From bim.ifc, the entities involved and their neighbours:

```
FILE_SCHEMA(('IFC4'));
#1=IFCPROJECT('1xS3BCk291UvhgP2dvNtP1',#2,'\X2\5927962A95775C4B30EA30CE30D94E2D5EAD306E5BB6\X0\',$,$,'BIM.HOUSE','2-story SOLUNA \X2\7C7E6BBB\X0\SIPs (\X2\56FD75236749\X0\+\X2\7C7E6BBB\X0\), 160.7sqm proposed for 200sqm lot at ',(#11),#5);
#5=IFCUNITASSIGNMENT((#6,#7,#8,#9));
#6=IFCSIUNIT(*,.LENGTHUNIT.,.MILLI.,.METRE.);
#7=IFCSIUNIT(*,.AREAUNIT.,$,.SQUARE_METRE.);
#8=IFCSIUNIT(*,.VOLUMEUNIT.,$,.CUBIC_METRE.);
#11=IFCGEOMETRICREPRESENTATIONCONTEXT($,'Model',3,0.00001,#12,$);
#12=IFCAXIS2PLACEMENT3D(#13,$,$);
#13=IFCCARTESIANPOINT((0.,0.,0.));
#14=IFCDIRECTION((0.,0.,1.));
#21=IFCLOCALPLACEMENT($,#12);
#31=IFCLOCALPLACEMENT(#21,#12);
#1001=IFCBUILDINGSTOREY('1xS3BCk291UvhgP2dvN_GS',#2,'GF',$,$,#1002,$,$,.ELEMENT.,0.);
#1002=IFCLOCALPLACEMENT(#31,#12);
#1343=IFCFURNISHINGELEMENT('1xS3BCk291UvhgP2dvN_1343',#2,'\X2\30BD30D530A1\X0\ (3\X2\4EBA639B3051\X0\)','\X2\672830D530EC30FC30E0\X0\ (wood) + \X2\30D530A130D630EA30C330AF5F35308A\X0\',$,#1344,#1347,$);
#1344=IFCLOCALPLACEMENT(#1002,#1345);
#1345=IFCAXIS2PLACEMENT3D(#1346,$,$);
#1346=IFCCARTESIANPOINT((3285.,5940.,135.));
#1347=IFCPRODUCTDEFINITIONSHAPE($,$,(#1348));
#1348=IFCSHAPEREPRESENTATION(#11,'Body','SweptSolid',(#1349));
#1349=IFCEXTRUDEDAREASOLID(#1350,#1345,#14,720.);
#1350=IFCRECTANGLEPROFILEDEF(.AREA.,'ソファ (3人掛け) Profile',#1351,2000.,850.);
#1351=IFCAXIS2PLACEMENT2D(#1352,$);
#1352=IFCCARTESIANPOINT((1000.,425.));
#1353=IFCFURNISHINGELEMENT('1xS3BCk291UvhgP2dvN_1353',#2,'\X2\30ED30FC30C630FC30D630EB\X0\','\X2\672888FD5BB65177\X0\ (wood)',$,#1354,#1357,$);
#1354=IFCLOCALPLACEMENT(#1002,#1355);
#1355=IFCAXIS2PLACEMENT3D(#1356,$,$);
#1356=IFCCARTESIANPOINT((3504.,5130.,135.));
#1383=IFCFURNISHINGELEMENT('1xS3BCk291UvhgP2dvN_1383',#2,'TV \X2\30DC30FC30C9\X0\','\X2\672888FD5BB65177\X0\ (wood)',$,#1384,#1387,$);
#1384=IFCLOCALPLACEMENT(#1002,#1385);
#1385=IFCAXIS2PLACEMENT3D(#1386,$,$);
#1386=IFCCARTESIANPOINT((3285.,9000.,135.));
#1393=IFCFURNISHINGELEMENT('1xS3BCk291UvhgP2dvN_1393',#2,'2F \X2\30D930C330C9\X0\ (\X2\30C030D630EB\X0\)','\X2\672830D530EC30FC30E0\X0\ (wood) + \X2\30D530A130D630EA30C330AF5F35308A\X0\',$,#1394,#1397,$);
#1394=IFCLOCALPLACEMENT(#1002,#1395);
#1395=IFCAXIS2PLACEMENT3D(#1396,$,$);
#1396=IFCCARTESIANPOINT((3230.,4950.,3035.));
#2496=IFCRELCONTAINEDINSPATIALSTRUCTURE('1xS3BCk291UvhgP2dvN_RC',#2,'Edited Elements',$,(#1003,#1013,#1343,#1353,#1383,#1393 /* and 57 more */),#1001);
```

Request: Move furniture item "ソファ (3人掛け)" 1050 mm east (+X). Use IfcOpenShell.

```python
import ifcopenshell
import ifcopenshell.api.geometry
import ifcopenshell.util.placement

model = ifcopenshell.open("bim.ifc")

item = model.by_guid("1xS3BCk291UvhgP2dvN_1343")
matrix = ifcopenshell.util.placement.get_local_placement(item.ObjectPlacement)
matrix[0, 3] += 1050.0
ifcopenshell.api.geometry.edit_object_placement(model, product=item, matrix=matrix, is_si=False)

print(ifcopenshell.util.placement.get_local_placement(item.ObjectPlacement).round(3) + 0.0)

model.write("bim_v2.ifc")
```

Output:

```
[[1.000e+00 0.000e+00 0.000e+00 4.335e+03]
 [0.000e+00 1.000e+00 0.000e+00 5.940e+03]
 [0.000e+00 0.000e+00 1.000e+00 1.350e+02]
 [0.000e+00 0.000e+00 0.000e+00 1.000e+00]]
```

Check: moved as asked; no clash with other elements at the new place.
